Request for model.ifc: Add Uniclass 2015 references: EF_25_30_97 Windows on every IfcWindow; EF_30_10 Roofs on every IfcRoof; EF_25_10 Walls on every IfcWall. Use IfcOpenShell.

First a look at what the model holds.

```python
import ifcopenshell

model = ifcopenshell.open("model.ifc")
print(model.schema)
print("classifications:", [c.Name for c in model.by_type("IfcClassification")])
for ifc_class in ("IfcDoor", "IfcRoof", "IfcStair", "IfcWall", "IfcWindow"):
    print(ifc_class, len(model.by_type(ifc_class)))
```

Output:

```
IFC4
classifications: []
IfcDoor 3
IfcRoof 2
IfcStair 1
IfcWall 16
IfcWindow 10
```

```python
import ifcopenshell
import ifcopenshell.api.classification

model = ifcopenshell.open("model.ifc")

system = ifcopenshell.api.classification.add_classification(model, classification="Uniclass 2015")

codes = {
    "IfcWindow": ("EF_25_30_97", "Windows"),
    "IfcRoof": ("EF_30_10", "Roofs"),
    "IfcWall": ("EF_25_10", "Walls"),
}
for ifc_class, (code, name) in codes.items():
    products = model.by_type(ifc_class)
    ifcopenshell.api.classification.add_reference(
        model, products=products, classification=system, identification=code, name=name
    )
    print(code, len(products))

model.write("model_v2.ifc")
```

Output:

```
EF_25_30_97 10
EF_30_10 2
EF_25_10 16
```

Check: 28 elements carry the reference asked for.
